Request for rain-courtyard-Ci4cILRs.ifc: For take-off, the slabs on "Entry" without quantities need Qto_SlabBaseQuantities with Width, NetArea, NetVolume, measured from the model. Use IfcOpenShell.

First a look at what the model holds.

```python
import ifcopenshell
import ifcopenshell.util.element
import ifcopenshell.util.unit

model = ifcopenshell.open("rain-courtyard-Ci4cILRs.ifc")
print(model.schema)
for unit_type in ("LENGTHUNIT", "AREAUNIT", "VOLUMEUNIT"):
    print(unit_type, ifcopenshell.util.unit.calculate_unit_scale(model, unit_type))
storey = next(s for s in model.by_type("IfcBuildingStorey") if s.Name == "Entry")
slabs = [e for e in ifcopenshell.util.element.get_decomposition(storey) if e.is_a("IfcSlab")]
for e in sorted(slabs, key=lambda e: e.id()):
    print(e.id(), e.is_a(), e.Name, list(ifcopenshell.util.element.get_psets(e, qtos_only=True)), sep=" | ")
```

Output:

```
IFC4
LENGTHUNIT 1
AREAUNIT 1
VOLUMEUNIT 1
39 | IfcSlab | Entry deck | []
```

```python
import ifcopenshell
import ifcopenshell.api.pset
import ifcopenshell.geom
import ifcopenshell.util.element
import ifcopenshell.util.shape
import ifcopenshell.util.unit

model = ifcopenshell.open("rain-courtyard-Ci4cILRs.ifc")
unit_scale = ifcopenshell.util.unit.calculate_unit_scale(model)
area_scale = ifcopenshell.util.unit.calculate_unit_scale(model, "AREAUNIT")
volume_scale = ifcopenshell.util.unit.calculate_unit_scale(model, "VOLUMEUNIT")
settings = ifcopenshell.geom.settings()

storey = next(s for s in model.by_type("IfcBuildingStorey") if s.Name == "Entry")
slabs = [e for e in ifcopenshell.util.element.get_decomposition(storey) if e.is_a("IfcSlab")]

for e in sorted(slabs, key=lambda e: e.id()):
    if ifcopenshell.util.element.get_psets(e, qtos_only=True, should_inherit=False):
        continue
    # Geometry comes back in metres, in the element's own axes.
    shape = ifcopenshell.geom.create_shape(settings, e)
    values = {
        "Width": ifcopenshell.util.shape.get_z(shape.geometry) / unit_scale,
        "NetArea": ifcopenshell.util.shape.get_footprint_area(shape.geometry) / area_scale,
        "NetVolume": ifcopenshell.util.shape.get_volume(shape.geometry) / volume_scale,
    }
    qto = ifcopenshell.api.pset.add_qto(model, product=e, name="Qto_SlabBaseQuantities")
    ifcopenshell.api.pset.edit_qto(model, qto=qto, properties=values)
    print(e.id(), {k: round(v, 3) for k, v in values.items()})

model.write("rain-courtyard-Ci4cILRs_v2.ifc")
```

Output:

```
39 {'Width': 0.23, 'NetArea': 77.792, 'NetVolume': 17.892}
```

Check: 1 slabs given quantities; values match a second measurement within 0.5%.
